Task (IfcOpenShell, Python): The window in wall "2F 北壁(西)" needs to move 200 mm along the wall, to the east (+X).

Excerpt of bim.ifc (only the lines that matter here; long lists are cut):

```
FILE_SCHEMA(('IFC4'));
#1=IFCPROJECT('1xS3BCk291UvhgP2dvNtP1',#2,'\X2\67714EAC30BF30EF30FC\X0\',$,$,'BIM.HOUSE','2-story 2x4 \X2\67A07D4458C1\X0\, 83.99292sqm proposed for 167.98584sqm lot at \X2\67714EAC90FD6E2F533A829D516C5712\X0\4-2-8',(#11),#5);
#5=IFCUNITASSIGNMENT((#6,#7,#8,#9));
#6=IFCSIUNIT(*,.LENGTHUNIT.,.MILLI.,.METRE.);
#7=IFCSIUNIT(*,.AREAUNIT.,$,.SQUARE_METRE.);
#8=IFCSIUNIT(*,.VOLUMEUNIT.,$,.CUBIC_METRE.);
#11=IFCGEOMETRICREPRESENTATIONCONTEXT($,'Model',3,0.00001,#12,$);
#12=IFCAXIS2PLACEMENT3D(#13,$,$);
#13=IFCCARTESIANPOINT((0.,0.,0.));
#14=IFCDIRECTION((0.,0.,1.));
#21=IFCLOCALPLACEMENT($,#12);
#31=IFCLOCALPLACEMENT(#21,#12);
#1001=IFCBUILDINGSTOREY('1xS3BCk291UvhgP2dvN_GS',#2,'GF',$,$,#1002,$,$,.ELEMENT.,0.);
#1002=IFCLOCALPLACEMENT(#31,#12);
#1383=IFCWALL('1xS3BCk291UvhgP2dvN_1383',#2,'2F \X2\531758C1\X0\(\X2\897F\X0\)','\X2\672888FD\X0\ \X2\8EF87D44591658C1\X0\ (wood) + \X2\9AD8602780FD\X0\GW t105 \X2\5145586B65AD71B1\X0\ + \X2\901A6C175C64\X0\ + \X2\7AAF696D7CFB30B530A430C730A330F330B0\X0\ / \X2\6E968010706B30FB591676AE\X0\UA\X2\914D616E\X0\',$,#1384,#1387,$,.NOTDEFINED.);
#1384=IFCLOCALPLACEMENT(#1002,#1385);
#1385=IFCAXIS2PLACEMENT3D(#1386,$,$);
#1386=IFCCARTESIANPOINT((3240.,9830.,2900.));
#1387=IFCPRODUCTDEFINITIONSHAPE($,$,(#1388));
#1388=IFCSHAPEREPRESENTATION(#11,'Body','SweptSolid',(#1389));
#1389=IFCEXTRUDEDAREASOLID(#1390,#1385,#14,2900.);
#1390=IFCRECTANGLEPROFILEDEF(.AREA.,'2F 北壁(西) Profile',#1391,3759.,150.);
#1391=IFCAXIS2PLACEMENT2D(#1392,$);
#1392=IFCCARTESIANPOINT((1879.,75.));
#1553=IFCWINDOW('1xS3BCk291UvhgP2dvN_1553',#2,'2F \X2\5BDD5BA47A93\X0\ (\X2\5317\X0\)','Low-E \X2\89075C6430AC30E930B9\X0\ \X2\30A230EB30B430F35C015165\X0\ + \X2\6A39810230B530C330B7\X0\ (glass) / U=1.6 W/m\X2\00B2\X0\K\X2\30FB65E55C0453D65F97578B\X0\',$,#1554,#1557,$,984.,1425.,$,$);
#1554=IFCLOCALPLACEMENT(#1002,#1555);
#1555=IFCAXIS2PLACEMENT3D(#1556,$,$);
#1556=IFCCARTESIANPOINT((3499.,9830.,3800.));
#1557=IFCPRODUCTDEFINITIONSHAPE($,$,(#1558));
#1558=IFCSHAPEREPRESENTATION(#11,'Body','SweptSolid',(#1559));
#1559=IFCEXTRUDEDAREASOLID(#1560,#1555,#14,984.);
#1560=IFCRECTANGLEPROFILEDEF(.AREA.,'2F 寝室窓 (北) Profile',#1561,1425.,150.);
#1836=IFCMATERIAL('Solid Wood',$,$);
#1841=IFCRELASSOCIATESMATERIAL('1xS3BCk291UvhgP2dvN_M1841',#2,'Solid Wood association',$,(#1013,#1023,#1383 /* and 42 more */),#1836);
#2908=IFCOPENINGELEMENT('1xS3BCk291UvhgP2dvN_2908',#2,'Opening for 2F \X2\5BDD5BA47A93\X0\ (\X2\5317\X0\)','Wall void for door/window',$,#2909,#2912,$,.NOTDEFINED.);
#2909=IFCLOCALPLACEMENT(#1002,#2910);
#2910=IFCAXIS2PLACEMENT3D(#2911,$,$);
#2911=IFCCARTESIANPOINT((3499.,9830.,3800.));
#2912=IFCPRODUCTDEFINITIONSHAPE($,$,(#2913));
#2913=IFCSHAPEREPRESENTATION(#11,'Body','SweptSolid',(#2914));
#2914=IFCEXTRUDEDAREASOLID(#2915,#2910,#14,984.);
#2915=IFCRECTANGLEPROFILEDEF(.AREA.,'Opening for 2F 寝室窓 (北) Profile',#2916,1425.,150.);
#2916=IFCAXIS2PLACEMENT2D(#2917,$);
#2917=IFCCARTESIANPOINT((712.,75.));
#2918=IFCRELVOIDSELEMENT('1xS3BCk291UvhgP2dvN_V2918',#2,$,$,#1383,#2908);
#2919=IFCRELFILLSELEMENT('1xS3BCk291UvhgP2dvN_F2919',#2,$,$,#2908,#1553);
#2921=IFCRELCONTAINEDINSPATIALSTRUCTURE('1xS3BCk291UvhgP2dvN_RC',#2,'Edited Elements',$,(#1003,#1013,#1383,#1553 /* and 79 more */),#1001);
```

```python
import ifcopenshell
import ifcopenshell.api.geometry
import ifcopenshell.util.placement
import ifcopenshell.util.unit

model = ifcopenshell.open("bim.ifc")
unit_scale = ifcopenshell.util.unit.calculate_unit_scale(model)

window = model.by_guid("1xS3BCk291UvhgP2dvN_1553")
opening = window.FillsVoids[0].RelatingOpeningElement
wall = opening.VoidsElements[0].RelatingBuildingElement

wall_matrix = ifcopenshell.util.placement.get_local_placement(wall.ObjectPlacement)
shift = wall_matrix[:3, 0] * 0.2 / unit_scale
before = ifcopenshell.util.placement.get_local_placement(window.ObjectPlacement)[:3, 3].copy()

# The window is not placed relative to its opening, so move both.
for product in (opening, window):
    matrix = ifcopenshell.util.placement.get_local_placement(product.ObjectPlacement)
    matrix[:3, 3] += shift
    ifcopenshell.api.geometry.edit_object_placement(model, product=product, matrix=matrix, is_si=False)

after = ifcopenshell.util.placement.get_local_placement(window.ObjectPlacement)[:3, 3]
print("window moved by", (after - before).round(3) + 0.0)

model.write("bim_rev.ifc")
```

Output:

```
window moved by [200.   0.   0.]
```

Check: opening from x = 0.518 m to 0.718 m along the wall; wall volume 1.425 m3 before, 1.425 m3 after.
